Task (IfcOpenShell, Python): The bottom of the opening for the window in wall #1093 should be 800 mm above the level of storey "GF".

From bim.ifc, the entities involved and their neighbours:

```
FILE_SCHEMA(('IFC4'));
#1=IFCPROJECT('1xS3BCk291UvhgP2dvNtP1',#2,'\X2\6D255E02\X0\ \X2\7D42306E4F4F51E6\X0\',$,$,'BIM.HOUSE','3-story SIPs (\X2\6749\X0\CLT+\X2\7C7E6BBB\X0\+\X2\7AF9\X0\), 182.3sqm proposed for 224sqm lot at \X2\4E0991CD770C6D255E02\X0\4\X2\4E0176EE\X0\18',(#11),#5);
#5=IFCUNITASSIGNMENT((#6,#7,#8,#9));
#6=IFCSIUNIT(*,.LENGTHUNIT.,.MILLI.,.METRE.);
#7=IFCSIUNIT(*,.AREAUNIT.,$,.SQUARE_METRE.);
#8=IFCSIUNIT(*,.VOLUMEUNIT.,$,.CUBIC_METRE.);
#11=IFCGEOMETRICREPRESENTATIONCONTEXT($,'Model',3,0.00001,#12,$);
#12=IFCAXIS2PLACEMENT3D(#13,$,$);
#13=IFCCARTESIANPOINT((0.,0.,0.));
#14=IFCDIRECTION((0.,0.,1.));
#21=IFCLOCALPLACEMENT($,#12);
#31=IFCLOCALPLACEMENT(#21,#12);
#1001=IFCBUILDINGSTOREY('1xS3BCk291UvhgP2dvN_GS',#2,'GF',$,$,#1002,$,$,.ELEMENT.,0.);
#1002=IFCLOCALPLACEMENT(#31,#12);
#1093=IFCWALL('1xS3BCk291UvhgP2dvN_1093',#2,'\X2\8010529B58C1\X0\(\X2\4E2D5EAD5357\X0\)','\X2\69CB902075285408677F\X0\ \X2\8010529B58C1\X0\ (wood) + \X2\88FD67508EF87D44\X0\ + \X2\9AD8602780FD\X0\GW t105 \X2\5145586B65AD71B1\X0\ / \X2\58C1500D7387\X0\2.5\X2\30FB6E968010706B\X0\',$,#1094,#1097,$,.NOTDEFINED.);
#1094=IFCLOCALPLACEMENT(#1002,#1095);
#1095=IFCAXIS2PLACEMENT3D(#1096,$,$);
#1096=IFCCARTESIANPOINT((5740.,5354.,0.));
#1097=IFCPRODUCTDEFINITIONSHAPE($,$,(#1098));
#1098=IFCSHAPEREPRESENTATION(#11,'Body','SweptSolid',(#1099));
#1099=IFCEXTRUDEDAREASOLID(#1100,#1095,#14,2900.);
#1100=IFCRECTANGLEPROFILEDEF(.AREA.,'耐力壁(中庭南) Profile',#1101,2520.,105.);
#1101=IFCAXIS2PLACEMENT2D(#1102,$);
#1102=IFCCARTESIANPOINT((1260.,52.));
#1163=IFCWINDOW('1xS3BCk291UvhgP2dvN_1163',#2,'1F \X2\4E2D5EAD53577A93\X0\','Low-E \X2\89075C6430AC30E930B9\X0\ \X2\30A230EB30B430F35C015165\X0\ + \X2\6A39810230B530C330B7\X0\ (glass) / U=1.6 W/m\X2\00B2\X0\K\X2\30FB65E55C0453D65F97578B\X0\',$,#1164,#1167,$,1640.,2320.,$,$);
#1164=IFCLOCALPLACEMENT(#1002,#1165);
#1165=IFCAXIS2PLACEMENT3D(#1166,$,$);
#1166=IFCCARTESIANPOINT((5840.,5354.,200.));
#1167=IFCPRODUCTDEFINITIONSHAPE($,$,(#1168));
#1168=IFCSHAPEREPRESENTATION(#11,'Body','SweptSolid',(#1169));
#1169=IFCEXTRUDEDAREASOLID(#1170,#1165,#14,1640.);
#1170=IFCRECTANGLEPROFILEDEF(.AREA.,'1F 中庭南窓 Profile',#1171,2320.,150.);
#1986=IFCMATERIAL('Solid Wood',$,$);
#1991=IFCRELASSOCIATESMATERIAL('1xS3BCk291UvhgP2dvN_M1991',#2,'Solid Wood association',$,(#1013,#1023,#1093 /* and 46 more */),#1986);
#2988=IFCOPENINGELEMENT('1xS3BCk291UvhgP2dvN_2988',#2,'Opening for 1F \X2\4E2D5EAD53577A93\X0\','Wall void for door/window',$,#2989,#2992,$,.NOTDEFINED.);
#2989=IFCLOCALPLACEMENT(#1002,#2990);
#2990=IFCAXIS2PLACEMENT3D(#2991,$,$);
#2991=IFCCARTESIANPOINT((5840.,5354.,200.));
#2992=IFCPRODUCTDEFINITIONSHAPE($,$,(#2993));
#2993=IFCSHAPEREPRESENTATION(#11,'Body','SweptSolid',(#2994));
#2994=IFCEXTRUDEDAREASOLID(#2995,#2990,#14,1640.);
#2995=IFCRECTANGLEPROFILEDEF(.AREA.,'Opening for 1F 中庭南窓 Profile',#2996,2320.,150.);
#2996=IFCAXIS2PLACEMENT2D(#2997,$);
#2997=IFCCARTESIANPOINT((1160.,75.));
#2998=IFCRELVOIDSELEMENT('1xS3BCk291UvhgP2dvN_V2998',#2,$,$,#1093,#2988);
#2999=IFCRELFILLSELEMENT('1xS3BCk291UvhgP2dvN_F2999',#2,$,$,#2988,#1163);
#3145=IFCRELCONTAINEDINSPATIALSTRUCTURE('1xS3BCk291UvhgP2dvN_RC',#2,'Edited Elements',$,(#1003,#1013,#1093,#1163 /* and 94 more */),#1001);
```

```python
import numpy as np
import ifcopenshell
import ifcopenshell.api.geometry
import ifcopenshell.geom
import ifcopenshell.util.element
import ifcopenshell.util.placement
import ifcopenshell.util.shape
import ifcopenshell.util.unit

model = ifcopenshell.open("bim.ifc")
unit_scale = ifcopenshell.util.unit.calculate_unit_scale(model)

window = model.by_id(1163)
opening = window.FillsVoids[0].RelatingOpeningElement
storey = ifcopenshell.util.element.get_container(window, ifc_class="IfcBuildingStorey")
level = ifcopenshell.util.placement.get_local_placement(storey.ObjectPlacement)[2, 3]

# The opening's origin need not be at the sill, so measure its lowest point.
shape = ifcopenshell.geom.create_shape(ifcopenshell.geom.settings(), opening)
bottom = ifcopenshell.util.shape.get_shape_bottom_elevation(shape, shape.geometry) / unit_scale
dz = level + 800.0 - bottom

shift = np.array([0.0, 0.0, dz])
# The window is not placed relative to its opening, so move both.
for product in (opening, window):
    matrix = ifcopenshell.util.placement.get_local_placement(product.ObjectPlacement)
    matrix[:3, 3] += shift
    ifcopenshell.api.geometry.edit_object_placement(model, product=product, matrix=matrix, is_si=False)

print(f"moved by {dz * unit_scale:+.3f} m")

model.write("bim_v2.ifc")
```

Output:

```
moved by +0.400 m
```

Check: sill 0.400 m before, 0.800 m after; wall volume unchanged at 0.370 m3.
